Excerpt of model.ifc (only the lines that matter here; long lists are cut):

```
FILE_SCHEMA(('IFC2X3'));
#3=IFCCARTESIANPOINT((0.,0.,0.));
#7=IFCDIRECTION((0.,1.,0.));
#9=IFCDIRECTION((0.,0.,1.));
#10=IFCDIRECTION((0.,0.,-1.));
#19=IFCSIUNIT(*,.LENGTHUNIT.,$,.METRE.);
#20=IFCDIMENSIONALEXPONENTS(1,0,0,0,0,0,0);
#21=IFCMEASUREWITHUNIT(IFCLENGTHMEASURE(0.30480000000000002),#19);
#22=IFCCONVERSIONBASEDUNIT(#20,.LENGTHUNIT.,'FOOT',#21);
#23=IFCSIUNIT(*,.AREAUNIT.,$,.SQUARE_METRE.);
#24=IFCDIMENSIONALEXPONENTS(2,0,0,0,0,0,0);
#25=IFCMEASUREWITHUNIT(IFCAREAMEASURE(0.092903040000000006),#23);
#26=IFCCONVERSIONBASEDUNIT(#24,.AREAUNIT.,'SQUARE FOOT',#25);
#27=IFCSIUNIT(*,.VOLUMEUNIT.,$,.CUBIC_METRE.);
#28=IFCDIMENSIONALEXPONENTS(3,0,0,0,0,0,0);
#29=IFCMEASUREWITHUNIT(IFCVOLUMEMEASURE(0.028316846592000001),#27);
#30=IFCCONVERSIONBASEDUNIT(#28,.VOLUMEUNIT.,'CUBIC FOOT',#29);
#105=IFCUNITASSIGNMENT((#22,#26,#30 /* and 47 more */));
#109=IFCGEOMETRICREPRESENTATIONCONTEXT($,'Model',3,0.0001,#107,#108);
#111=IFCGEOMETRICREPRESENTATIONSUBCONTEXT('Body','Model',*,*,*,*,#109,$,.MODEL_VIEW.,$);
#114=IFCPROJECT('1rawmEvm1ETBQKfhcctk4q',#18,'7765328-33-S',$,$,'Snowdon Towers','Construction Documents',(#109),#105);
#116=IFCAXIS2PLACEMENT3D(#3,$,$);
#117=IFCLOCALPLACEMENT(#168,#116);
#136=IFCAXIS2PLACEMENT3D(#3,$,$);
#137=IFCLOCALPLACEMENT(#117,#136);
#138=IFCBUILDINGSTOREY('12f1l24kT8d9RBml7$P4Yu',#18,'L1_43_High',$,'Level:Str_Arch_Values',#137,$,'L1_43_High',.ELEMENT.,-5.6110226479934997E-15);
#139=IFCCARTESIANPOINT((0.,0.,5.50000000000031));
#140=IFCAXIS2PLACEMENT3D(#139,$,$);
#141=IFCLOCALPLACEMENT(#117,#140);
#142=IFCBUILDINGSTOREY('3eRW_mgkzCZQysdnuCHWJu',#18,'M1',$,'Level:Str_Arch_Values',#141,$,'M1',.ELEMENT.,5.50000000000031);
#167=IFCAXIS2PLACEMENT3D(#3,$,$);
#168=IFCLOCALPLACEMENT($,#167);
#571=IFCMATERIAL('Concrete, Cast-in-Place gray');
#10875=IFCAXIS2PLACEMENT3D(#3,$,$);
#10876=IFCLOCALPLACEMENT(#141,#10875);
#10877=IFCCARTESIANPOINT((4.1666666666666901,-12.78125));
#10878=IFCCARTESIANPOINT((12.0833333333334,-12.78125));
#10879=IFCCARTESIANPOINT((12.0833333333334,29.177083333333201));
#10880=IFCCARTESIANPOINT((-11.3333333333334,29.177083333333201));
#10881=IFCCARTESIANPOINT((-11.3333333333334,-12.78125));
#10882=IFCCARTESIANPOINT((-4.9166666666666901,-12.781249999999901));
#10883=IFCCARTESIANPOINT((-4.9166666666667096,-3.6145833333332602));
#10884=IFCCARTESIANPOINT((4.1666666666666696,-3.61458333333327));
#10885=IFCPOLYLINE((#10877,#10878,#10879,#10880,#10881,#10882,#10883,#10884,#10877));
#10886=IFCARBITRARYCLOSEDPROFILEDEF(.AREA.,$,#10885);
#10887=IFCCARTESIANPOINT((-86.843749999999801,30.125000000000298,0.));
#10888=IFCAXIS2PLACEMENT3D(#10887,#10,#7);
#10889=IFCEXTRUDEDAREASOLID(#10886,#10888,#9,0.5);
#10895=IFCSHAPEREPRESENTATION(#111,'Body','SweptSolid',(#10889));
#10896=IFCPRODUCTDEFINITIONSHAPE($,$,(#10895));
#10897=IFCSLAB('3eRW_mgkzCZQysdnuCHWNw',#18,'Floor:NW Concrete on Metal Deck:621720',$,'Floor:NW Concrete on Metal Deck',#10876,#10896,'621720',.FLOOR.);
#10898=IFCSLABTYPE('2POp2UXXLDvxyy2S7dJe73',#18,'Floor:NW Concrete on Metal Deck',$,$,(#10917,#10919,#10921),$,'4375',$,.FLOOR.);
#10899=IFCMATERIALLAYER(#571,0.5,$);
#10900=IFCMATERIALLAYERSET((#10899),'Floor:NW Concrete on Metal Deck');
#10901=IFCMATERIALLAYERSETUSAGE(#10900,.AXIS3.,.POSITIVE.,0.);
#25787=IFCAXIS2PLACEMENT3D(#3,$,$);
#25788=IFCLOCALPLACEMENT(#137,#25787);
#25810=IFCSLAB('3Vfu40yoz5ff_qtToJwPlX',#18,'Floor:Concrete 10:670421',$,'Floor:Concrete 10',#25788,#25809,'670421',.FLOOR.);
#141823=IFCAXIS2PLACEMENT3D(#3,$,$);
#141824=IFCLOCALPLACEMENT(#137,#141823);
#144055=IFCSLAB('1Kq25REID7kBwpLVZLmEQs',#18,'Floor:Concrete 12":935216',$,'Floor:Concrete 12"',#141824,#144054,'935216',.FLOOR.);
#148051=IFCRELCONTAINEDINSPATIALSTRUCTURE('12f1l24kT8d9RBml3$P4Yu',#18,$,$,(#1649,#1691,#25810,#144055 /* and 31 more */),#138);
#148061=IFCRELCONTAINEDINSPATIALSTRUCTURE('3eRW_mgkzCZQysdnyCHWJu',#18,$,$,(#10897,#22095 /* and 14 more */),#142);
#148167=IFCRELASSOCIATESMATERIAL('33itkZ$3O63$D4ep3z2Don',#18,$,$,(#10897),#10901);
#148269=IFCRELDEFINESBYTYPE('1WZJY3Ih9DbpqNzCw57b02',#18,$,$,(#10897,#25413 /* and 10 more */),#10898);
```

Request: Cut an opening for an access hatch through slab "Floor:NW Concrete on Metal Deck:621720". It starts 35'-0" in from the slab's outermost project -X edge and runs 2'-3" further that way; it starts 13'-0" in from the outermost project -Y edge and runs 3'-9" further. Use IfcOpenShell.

```python
import numpy as np
import ifcopenshell
import ifcopenshell.api.feature
import ifcopenshell.api.geometry
import ifcopenshell.api.root
import ifcopenshell.geom
import ifcopenshell.util.placement
import ifcopenshell.util.representation
import ifcopenshell.util.shape
import ifcopenshell.util.unit

model = ifcopenshell.open("model.ifc")
unit_scale = ifcopenshell.util.unit.calculate_unit_scale(model)
settings = ifcopenshell.geom.settings()


def volume(element):
    """Net volume in cubic metres, openings subtracted."""
    shape = ifcopenshell.geom.create_shape(settings, element)
    return ifcopenshell.util.shape.get_volume(shape.geometry)


slab = model.by_id(10897)
before = volume(slab)

# Extent in the slab's own axes, in metres. The edges named are its -X and -Y sides.
slab_shape = ifcopenshell.geom.create_shape(settings, slab)
vertices = ifcopenshell.util.shape.get_vertices(slab_shape.geometry)
x_min, y_min, bottom = vertices.min(axis=0)
top = vertices[:, 2].max()

opening = ifcopenshell.api.root.create_entity(model, ifc_class="IfcOpeningElement", name="Access hatch opening")
context = ifcopenshell.util.representation.get_context(model, "Model", "Body", "MODEL_VIEW")
width, depth = 0.6858, 1.143
outline = [(0.0, 0.0), (width, 0.0), (width, depth), (0.0, depth), (0.0, 0.0)]
# Overshoot both faces by 50 mm so the cut is clean.
shape = ifcopenshell.api.geometry.add_slab_representation(
    model, context=context, depth=top - bottom + 0.1, polyline=outline
)
ifcopenshell.api.geometry.assign_representation(model, product=opening, representation=shape)

matrix = ifcopenshell.util.placement.get_local_placement(slab.ObjectPlacement)
matrix[:, 3] = matrix @ np.append(np.array([x_min + 10.668, y_min + 3.9624, bottom - 0.05]) / unit_scale, 1.0)
ifcopenshell.api.geometry.edit_object_placement(model, product=opening, matrix=matrix, is_si=False)
ifcopenshell.api.feature.add_feature(model, feature=opening, element=slab)

after = volume(slab)

print(f"slab volume {before:.3f} -> {after:.3f} m3")

model.write("model_v2.ifc")
```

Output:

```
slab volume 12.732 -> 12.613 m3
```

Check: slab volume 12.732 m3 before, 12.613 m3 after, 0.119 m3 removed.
